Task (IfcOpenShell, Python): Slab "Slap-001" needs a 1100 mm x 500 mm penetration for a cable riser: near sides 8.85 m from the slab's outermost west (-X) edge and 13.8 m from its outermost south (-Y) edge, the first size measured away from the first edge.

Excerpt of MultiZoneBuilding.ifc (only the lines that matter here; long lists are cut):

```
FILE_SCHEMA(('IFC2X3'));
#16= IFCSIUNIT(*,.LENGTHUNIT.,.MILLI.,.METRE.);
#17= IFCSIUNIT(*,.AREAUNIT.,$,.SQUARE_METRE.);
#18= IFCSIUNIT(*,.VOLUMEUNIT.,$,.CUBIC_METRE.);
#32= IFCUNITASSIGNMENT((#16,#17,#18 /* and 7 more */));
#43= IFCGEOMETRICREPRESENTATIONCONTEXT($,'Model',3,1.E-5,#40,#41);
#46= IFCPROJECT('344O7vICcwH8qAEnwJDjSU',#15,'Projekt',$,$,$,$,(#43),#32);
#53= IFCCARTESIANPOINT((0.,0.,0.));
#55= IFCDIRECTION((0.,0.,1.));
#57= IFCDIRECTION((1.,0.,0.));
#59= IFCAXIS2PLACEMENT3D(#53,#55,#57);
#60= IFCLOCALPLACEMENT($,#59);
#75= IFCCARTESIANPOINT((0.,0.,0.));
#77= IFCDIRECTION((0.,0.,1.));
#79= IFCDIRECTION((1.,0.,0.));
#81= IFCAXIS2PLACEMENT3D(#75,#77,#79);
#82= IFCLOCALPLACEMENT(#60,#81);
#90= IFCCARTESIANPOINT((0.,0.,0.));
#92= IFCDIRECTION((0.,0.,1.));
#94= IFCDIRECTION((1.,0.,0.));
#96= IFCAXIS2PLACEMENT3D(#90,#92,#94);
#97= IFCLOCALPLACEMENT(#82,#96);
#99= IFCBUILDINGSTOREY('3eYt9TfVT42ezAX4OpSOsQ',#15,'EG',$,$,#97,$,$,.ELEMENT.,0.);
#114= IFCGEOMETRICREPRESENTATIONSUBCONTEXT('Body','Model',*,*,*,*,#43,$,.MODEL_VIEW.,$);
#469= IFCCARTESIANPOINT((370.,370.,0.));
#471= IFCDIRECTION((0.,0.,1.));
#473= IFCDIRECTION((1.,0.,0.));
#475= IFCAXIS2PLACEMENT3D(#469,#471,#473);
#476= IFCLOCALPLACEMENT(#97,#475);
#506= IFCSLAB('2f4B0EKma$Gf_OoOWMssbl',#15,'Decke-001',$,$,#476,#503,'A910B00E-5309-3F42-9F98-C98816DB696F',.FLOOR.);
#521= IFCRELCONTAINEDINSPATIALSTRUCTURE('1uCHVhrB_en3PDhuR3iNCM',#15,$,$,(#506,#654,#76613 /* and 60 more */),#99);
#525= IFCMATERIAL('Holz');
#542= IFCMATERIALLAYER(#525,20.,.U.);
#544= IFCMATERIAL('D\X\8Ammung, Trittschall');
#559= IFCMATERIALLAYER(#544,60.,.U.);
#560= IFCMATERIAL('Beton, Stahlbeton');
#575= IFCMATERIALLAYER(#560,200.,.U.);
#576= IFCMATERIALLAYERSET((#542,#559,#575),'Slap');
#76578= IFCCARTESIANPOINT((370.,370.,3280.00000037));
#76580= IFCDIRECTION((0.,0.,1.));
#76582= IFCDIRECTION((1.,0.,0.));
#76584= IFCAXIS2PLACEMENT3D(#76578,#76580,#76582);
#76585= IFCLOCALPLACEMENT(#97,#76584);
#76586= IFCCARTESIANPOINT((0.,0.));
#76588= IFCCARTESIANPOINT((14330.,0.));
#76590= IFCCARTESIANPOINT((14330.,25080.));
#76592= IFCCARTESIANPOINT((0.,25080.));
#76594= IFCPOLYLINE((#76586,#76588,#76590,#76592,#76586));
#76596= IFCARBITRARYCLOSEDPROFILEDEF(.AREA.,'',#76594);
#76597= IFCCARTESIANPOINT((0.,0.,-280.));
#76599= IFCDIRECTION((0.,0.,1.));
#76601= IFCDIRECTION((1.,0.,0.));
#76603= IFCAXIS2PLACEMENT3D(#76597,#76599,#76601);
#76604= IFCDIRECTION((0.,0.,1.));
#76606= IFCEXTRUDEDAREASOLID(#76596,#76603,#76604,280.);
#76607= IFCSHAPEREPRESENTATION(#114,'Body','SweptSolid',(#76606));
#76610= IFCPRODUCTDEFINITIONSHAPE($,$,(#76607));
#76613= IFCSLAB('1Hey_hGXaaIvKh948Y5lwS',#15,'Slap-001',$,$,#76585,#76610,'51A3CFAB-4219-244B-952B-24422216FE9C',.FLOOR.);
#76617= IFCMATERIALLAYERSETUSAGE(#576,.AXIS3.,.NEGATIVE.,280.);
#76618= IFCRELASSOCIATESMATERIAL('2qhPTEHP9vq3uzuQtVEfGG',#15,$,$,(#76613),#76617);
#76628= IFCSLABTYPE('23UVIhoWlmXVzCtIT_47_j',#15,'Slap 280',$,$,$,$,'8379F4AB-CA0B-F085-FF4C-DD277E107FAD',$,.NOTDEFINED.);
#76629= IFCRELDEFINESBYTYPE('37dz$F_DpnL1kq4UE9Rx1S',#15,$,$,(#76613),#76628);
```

```python
import numpy as np
import ifcopenshell
import ifcopenshell.api.feature
import ifcopenshell.api.geometry
import ifcopenshell.api.root
import ifcopenshell.geom
import ifcopenshell.util.placement
import ifcopenshell.util.representation
import ifcopenshell.util.shape
import ifcopenshell.util.unit

model = ifcopenshell.open("MultiZoneBuilding.ifc")
unit_scale = ifcopenshell.util.unit.calculate_unit_scale(model)
settings = ifcopenshell.geom.settings()


def volume(element):
    """Net volume in cubic metres, openings subtracted."""
    shape = ifcopenshell.geom.create_shape(settings, element)
    return ifcopenshell.util.shape.get_volume(shape.geometry)


slab = model.by_guid("1Hey_hGXaaIvKh948Y5lwS")
before = volume(slab)

# Extent in the slab's own axes, in metres. The edges named are its -X and -Y sides.
slab_shape = ifcopenshell.geom.create_shape(settings, slab)
vertices = ifcopenshell.util.shape.get_vertices(slab_shape.geometry)
x_min, y_min, bottom = vertices.min(axis=0)
top = vertices[:, 2].max()

opening = ifcopenshell.api.root.create_entity(model, ifc_class="IfcOpeningElement", name="Cable riser opening")
context = ifcopenshell.util.representation.get_context(model, "Model", "Body", "MODEL_VIEW")
width, depth = 1.1, 0.5
outline = [(0.0, 0.0), (width, 0.0), (width, depth), (0.0, depth), (0.0, 0.0)]
# Overshoot both faces by 50 mm so the cut is clean.
shape = ifcopenshell.api.geometry.add_slab_representation(
    model, context=context, depth=top - bottom + 0.1, polyline=outline
)
ifcopenshell.api.geometry.assign_representation(model, product=opening, representation=shape)

matrix = ifcopenshell.util.placement.get_local_placement(slab.ObjectPlacement)
matrix[:, 3] = matrix @ np.append(np.array([x_min + 8.85, y_min + 13.8, bottom - 0.05]) / unit_scale, 1.0)
ifcopenshell.api.geometry.edit_object_placement(model, product=opening, matrix=matrix, is_si=False)
ifcopenshell.api.feature.add_feature(model, feature=opening, element=slab)

after = volume(slab)

print(f"slab volume {before:.3f} -> {after:.3f} m3")

model.write("MultiZoneBuilding_updated.ifc")
```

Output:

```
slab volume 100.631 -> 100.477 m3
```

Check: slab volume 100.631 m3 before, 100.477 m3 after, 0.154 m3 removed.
